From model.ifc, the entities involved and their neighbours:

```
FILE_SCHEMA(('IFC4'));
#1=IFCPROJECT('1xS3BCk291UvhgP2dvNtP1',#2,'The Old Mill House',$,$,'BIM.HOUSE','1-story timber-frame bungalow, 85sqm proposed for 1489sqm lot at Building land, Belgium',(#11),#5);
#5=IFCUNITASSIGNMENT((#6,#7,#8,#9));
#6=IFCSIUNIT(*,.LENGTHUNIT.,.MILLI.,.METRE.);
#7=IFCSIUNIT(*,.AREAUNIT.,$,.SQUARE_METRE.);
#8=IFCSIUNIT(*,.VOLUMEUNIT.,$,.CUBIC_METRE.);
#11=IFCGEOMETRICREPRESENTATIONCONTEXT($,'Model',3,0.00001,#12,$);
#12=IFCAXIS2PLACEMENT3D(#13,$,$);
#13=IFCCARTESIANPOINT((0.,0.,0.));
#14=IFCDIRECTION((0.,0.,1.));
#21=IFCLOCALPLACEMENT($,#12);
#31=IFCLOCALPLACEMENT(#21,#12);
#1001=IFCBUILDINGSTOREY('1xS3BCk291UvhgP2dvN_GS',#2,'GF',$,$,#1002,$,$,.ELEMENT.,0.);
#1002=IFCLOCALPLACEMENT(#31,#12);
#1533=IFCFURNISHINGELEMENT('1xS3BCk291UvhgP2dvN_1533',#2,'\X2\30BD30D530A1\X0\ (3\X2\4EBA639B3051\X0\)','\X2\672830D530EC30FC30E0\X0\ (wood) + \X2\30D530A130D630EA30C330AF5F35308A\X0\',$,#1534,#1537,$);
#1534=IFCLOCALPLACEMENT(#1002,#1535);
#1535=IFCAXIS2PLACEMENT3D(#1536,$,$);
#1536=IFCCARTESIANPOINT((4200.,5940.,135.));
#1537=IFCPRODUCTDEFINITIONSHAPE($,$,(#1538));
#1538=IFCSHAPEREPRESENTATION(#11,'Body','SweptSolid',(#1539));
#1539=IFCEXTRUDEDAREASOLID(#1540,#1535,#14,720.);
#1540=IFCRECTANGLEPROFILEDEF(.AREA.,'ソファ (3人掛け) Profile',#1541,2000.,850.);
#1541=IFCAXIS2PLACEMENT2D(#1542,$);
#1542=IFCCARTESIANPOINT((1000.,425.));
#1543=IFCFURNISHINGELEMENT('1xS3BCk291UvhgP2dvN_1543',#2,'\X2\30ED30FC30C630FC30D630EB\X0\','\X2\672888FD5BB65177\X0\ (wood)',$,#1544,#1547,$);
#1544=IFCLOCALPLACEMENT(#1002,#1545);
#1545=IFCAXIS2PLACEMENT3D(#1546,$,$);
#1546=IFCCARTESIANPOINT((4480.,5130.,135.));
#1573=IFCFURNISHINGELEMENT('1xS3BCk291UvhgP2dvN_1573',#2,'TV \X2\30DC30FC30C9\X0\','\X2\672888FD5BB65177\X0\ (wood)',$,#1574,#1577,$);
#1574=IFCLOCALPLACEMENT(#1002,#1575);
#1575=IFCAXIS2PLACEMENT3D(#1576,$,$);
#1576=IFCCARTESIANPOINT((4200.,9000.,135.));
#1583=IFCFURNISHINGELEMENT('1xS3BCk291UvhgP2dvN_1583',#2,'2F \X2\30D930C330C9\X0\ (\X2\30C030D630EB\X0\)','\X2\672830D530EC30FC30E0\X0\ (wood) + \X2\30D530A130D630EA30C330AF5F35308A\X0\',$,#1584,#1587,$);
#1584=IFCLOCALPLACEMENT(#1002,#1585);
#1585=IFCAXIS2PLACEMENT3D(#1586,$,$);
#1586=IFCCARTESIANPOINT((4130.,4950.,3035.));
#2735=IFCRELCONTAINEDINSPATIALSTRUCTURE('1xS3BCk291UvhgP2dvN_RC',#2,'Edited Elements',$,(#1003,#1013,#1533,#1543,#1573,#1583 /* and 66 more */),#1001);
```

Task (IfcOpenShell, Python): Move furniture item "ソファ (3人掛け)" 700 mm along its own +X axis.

```python
import ifcopenshell
import ifcopenshell.api.geometry
import ifcopenshell.util.placement

model = ifcopenshell.open("model.ifc")

item = model.by_guid("1xS3BCk291UvhgP2dvN_1533")
matrix = ifcopenshell.util.placement.get_local_placement(item.ObjectPlacement)
matrix[:3, 3] += matrix[:3, 0] * 700.0
ifcopenshell.api.geometry.edit_object_placement(model, product=item, matrix=matrix, is_si=False)

print(ifcopenshell.util.placement.get_local_placement(item.ObjectPlacement).round(3) + 0.0)

model.write("model_edited.ifc")
```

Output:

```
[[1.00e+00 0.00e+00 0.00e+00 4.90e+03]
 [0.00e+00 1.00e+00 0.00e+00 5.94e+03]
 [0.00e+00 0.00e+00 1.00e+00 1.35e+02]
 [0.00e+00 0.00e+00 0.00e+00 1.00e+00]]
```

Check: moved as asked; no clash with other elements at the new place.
